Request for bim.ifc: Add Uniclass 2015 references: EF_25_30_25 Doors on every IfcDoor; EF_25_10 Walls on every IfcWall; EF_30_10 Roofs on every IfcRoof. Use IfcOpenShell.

First a look at what the model holds.

```python
import ifcopenshell

model = ifcopenshell.open("bim.ifc")
print(model.schema)
print("classifications:", [c.Name for c in model.by_type("IfcClassification")])
for ifc_class in ("IfcDoor", "IfcRoof", "IfcStair", "IfcWall", "IfcWindow"):
    print(ifc_class, len(model.by_type(ifc_class)))
```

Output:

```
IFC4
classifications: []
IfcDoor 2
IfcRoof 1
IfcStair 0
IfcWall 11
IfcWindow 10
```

```python
import ifcopenshell
import ifcopenshell.api.classification

model = ifcopenshell.open("bim.ifc")

system = ifcopenshell.api.classification.add_classification(model, classification="Uniclass 2015")

codes = {
    "IfcDoor": ("EF_25_30_25", "Doors"),
    "IfcWall": ("EF_25_10", "Walls"),
    "IfcRoof": ("EF_30_10", "Roofs"),
}
for ifc_class, (code, name) in codes.items():
    products = model.by_type(ifc_class)
    ifcopenshell.api.classification.add_reference(
        model, products=products, classification=system, identification=code, name=name
    )
    print(code, len(products))

model.write("bim-out.ifc")
```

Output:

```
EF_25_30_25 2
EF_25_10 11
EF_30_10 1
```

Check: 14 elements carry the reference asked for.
